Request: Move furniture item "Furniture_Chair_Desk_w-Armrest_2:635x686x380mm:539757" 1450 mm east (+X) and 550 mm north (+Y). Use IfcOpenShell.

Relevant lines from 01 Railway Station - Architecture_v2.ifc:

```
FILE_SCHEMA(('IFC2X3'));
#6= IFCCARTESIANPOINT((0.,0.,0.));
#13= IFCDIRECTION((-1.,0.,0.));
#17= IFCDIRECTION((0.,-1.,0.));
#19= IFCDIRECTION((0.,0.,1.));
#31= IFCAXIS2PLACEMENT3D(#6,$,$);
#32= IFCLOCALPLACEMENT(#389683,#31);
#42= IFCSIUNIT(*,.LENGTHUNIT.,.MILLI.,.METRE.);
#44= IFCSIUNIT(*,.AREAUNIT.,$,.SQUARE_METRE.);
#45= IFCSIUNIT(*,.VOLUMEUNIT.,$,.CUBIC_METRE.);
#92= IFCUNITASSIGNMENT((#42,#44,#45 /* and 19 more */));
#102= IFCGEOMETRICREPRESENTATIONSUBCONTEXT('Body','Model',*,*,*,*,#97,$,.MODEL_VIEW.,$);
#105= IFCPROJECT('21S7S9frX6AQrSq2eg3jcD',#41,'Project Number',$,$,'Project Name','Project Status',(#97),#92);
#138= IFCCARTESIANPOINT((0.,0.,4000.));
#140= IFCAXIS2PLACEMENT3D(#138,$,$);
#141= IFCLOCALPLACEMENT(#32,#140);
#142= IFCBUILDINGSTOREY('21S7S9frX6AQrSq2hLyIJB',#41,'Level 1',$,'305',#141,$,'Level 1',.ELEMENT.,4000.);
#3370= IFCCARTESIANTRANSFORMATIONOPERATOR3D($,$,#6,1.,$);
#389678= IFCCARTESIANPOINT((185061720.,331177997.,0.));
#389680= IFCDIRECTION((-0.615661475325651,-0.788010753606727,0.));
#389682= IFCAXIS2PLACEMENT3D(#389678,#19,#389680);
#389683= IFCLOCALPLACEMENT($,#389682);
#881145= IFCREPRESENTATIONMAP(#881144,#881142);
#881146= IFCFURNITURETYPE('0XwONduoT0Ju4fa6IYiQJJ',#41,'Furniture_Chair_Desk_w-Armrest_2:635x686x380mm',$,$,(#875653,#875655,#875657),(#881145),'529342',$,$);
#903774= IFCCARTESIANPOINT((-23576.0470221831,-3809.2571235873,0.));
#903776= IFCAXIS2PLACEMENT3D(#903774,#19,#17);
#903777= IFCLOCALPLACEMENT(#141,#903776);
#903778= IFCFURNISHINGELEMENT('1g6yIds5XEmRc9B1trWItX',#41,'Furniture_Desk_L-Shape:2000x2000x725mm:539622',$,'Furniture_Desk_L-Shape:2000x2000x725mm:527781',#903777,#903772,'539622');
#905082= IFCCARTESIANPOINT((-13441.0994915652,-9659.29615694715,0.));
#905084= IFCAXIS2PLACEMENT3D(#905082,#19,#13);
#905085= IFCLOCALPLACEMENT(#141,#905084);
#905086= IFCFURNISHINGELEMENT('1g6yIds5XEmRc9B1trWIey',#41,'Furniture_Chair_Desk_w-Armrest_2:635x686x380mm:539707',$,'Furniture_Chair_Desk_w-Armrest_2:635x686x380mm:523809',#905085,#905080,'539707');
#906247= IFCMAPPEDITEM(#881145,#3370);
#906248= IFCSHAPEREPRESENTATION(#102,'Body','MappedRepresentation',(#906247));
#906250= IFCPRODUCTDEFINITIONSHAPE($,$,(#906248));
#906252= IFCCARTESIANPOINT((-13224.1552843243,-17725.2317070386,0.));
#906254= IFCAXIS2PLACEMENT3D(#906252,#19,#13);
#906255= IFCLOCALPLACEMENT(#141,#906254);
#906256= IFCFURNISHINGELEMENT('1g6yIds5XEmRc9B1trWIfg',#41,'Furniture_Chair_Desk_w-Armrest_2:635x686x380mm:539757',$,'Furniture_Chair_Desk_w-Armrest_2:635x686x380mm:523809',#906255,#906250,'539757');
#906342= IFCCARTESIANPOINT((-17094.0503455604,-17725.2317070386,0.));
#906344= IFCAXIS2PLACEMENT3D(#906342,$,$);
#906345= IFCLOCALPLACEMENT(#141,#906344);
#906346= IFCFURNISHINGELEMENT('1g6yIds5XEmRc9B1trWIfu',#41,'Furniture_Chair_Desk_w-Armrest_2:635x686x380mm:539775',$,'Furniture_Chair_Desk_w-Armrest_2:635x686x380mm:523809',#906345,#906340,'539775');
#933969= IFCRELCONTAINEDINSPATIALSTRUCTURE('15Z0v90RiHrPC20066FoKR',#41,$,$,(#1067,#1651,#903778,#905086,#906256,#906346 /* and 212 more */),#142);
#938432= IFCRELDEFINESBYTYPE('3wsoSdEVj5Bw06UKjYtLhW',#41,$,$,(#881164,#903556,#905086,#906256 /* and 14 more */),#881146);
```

```python
import ifcopenshell
import ifcopenshell.api.geometry
import ifcopenshell.util.placement
import ifcopenshell.util.unit

model = ifcopenshell.open("01 Railway Station - Architecture_v2.ifc")
unit_scale = ifcopenshell.util.unit.calculate_unit_scale(model)

item = model.by_guid("1g6yIds5XEmRc9B1trWIfg")
matrix = ifcopenshell.util.placement.get_local_placement(item.ObjectPlacement)
matrix[0, 3] += 1.45 / unit_scale
matrix[1, 3] += 0.55 / unit_scale
ifcopenshell.api.geometry.edit_object_placement(model, product=item, matrix=matrix, is_si=False)

print(ifcopenshell.util.placement.get_local_placement(item.ObjectPlacement).round(3) + 0.0)

model.write("01 Railway Station - Architecture_v2-out.ifc")
```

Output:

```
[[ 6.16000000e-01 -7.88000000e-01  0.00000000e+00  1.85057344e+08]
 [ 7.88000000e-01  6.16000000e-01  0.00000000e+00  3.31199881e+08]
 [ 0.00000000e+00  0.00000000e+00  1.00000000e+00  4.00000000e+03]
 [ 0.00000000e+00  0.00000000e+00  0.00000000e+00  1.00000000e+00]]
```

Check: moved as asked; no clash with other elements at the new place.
